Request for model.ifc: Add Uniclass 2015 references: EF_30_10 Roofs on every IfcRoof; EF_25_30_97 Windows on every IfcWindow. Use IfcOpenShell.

First a look at what the model holds.

```python
import ifcopenshell

model = ifcopenshell.open("model.ifc")
print(model.schema)
print("classifications:", [c.Name for c in model.by_type("IfcClassification")])
for ifc_class in ("IfcDoor", "IfcRoof", "IfcStair", "IfcWall", "IfcWindow"):
    print(ifc_class, len(model.by_type(ifc_class)))
```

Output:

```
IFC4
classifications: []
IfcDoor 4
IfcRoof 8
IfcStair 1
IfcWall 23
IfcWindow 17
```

```python
import ifcopenshell
import ifcopenshell.api.classification

model = ifcopenshell.open("model.ifc")

system = ifcopenshell.api.classification.add_classification(model, classification="Uniclass 2015")

codes = {
    "IfcRoof": ("EF_30_10", "Roofs"),
    "IfcWindow": ("EF_25_30_97", "Windows"),
}
for ifc_class, (code, name) in codes.items():
    products = model.by_type(ifc_class)
    ifcopenshell.api.classification.add_reference(
        model, products=products, classification=system, identification=code, name=name
    )
    print(code, len(products))

model.write("model_rev.ifc")
```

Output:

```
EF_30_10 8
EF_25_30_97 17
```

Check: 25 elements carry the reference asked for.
